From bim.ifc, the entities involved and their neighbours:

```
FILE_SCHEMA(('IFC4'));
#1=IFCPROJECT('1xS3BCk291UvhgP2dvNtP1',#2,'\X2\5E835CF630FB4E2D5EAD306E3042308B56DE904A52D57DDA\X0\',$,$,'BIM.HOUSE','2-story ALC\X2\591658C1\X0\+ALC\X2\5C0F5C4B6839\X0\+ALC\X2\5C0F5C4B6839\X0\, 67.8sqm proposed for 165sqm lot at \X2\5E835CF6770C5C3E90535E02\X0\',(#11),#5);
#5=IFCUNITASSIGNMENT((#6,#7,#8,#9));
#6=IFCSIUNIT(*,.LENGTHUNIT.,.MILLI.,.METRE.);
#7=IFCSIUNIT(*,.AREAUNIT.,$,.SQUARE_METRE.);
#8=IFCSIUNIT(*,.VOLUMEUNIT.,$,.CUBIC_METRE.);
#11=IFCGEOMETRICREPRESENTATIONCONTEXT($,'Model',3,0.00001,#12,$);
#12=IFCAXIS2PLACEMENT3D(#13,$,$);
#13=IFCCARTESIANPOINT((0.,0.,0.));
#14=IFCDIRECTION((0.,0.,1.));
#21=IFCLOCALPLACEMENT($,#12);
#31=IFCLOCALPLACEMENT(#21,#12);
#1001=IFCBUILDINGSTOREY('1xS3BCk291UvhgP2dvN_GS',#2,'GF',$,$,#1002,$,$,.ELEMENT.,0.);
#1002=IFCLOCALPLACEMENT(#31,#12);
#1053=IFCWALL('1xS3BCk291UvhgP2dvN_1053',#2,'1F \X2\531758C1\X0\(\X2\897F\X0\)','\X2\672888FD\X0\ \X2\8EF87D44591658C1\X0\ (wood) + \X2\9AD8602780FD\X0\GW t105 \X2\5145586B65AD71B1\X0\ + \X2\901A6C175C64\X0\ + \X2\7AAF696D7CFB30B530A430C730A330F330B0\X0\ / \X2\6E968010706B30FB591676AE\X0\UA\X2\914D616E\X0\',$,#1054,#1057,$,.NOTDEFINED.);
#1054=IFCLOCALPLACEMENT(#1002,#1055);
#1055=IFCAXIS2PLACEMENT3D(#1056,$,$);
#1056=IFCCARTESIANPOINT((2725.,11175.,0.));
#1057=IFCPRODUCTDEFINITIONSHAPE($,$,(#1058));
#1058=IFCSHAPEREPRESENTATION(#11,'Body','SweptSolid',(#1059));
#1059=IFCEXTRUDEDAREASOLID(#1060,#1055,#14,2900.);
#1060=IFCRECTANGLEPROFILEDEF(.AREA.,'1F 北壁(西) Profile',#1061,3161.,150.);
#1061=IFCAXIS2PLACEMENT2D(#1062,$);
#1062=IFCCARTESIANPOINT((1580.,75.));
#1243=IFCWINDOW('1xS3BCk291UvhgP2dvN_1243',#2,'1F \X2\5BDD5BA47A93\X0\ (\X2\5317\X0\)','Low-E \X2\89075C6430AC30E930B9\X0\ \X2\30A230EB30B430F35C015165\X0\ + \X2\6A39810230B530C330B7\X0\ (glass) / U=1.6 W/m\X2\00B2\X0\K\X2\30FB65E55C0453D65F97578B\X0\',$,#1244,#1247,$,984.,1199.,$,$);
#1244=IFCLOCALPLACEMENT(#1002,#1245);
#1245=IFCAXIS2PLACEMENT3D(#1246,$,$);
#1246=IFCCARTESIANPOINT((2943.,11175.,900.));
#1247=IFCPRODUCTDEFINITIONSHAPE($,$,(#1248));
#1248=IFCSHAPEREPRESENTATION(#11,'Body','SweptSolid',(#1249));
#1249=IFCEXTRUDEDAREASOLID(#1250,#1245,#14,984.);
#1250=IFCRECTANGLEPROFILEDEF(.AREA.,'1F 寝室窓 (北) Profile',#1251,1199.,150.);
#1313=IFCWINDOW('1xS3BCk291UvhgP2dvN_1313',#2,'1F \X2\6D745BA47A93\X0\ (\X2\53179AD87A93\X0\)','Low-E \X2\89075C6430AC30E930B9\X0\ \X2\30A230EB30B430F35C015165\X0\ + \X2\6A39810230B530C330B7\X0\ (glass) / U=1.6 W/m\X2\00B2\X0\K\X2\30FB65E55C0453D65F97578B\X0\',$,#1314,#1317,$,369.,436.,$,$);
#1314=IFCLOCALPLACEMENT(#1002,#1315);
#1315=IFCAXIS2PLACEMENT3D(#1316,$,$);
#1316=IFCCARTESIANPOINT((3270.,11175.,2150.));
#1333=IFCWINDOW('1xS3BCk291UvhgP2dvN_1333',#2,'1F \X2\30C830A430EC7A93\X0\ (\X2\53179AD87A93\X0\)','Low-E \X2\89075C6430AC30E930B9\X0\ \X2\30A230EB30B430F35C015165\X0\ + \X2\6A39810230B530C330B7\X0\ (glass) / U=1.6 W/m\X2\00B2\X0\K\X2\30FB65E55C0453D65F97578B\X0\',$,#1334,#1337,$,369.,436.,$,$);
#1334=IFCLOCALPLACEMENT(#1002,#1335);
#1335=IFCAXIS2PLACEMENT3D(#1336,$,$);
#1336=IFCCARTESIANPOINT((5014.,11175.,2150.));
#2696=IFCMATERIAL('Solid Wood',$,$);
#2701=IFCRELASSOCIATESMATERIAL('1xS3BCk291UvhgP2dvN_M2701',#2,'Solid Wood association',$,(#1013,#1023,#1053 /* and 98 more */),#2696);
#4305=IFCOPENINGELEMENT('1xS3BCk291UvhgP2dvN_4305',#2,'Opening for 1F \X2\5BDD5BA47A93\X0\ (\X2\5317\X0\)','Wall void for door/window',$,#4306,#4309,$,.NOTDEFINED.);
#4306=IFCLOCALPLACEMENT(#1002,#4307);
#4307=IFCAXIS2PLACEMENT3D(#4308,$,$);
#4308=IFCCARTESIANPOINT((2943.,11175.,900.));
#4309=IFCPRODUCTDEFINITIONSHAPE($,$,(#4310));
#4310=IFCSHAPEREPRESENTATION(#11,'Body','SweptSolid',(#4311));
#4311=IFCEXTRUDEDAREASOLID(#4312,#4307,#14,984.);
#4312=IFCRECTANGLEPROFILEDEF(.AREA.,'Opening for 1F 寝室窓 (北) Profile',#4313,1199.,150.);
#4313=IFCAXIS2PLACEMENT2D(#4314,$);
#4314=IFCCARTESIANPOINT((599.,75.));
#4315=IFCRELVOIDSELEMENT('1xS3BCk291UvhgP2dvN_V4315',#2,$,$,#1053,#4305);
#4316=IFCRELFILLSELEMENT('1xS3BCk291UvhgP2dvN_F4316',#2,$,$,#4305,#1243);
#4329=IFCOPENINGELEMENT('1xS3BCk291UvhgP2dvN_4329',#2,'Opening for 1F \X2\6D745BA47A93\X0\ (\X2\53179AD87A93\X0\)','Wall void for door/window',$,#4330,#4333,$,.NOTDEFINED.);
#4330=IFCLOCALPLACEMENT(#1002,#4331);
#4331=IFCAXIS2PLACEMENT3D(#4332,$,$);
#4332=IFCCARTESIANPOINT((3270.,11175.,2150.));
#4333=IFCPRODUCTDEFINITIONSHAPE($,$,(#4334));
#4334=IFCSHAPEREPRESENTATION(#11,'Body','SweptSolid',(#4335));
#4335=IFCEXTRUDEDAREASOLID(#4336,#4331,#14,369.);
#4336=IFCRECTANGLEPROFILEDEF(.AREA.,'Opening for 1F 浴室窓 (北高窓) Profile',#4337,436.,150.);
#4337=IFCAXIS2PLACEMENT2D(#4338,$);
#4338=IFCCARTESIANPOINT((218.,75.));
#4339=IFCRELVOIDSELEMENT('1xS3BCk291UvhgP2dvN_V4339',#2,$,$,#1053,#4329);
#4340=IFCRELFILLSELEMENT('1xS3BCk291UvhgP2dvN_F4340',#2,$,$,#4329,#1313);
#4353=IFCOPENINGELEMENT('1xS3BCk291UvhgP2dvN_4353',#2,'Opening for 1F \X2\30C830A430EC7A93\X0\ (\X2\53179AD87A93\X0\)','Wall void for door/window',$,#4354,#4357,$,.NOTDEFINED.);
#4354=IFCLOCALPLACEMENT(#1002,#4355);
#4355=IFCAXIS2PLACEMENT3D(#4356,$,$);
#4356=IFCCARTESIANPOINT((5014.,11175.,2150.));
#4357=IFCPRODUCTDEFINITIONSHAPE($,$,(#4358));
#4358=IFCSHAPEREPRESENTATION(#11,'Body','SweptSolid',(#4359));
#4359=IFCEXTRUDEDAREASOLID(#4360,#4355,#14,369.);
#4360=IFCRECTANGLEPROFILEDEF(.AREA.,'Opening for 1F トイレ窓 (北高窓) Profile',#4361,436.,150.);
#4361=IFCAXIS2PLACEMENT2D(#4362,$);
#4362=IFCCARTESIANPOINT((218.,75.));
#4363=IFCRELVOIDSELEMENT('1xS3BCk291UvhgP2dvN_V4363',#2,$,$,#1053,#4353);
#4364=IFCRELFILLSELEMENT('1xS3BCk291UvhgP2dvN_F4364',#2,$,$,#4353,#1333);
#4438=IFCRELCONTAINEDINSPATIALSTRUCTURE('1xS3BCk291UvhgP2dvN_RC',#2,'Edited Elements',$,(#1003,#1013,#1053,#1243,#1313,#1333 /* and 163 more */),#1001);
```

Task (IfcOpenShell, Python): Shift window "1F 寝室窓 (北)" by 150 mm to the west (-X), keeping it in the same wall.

```python
import ifcopenshell
import ifcopenshell.api.geometry
import ifcopenshell.util.placement
import ifcopenshell.util.unit

model = ifcopenshell.open("bim.ifc")
unit_scale = ifcopenshell.util.unit.calculate_unit_scale(model)

window = model.by_id(1243)
opening = window.FillsVoids[0].RelatingOpeningElement
wall = opening.VoidsElements[0].RelatingBuildingElement

wall_matrix = ifcopenshell.util.placement.get_local_placement(wall.ObjectPlacement)
shift = wall_matrix[:3, 0] * -0.15 / unit_scale
before = ifcopenshell.util.placement.get_local_placement(window.ObjectPlacement)[:3, 3].copy()

# The window is not placed relative to its opening, so move both.
for product in (opening, window):
    matrix = ifcopenshell.util.placement.get_local_placement(product.ObjectPlacement)
    matrix[:3, 3] += shift
    ifcopenshell.api.geometry.edit_object_placement(model, product=product, matrix=matrix, is_si=False)

after = ifcopenshell.util.placement.get_local_placement(window.ObjectPlacement)[:3, 3]
print("window moved by", (after - before).round(3) + 0.0)

model.write("bim_rev.ifc")
```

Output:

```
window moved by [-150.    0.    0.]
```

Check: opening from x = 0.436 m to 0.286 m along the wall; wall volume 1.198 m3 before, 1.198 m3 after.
